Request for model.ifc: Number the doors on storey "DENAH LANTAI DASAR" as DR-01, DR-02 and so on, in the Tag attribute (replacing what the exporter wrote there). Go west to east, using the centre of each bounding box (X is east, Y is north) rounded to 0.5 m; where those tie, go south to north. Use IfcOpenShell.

First a look at what the model holds.

```python
import ifcopenshell
import ifcopenshell.util.element
import ifcopenshell.util.placement

model = ifcopenshell.open("model.ifc")
print(model.schema)
storey = next(s for s in model.by_type("IfcBuildingStorey") if s.Name == "DENAH LANTAI DASAR")
doors = [e for e in ifcopenshell.util.element.get_decomposition(storey) if e.is_a("IfcDoor")]
for e in sorted(doors, key=lambda e: e.id()):
    origin = ifcopenshell.util.placement.get_local_placement(e.ObjectPlacement)[:3, 3]
    print(e.id(), e.Tag, e.Name, origin.round(2) + 0.0, sep=" | ")
```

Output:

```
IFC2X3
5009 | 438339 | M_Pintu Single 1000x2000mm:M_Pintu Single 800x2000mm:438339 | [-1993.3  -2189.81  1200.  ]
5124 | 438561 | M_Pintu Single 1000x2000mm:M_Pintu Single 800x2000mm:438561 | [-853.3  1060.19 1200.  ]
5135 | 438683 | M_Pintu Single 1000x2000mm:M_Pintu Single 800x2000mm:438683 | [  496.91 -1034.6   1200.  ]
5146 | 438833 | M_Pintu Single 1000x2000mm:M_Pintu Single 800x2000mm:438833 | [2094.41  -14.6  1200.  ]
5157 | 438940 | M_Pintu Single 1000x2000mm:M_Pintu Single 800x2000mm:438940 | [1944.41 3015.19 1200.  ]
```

```python
import ifcopenshell
import ifcopenshell.geom
import ifcopenshell.util.element
import ifcopenshell.util.shape

model = ifcopenshell.open("model.ifc")
settings = ifcopenshell.geom.settings()
settings.set("use-world-coords", True)


def centre(element):
    shape = ifcopenshell.geom.create_shape(settings, element)
    return ifcopenshell.util.shape.get_bbox_centroid(shape.geometry)


storey = next(s for s in model.by_type("IfcBuildingStorey") if s.Name == "DENAH LANTAI DASAR")
doors = [e for e in ifcopenshell.util.element.get_decomposition(storey) if e.is_a("IfcDoor")]

# Insertion points can sit at a corner or the storey origin, so sort by the geometry (in metres).
centres = {e: centre(e) for e in doors}
doors.sort(key=lambda e: (round(centres[e][0] / 0.5), centres[e][1]))

for i, e in enumerate(doors, start=1):
    number = f"DR-{i:02d}"
    e.Tag = number
    print(e.id(), number)

model.write("model_edited.ifc")
```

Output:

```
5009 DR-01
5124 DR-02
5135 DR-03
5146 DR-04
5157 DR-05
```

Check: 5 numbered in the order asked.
